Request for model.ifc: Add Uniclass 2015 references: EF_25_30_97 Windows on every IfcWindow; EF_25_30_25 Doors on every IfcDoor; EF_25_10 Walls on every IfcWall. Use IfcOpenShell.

First a look at what the model holds.

```python
import ifcopenshell

model = ifcopenshell.open("model.ifc")
print(model.schema)
print("classifications:", [c.Name for c in model.by_type("IfcClassification")])
for ifc_class in ("IfcDoor", "IfcRoof", "IfcStair", "IfcWall", "IfcWindow"):
    print(ifc_class, len(model.by_type(ifc_class)))
```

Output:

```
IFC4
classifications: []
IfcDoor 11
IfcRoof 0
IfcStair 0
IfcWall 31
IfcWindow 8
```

```python
import ifcopenshell
import ifcopenshell.api.classification

model = ifcopenshell.open("model.ifc")

system = ifcopenshell.api.classification.add_classification(model, classification="Uniclass 2015")

codes = {
    "IfcWindow": ("EF_25_30_97", "Windows"),
    "IfcDoor": ("EF_25_30_25", "Doors"),
    "IfcWall": ("EF_25_10", "Walls"),
}
for ifc_class, (code, name) in codes.items():
    products = model.by_type(ifc_class)
    ifcopenshell.api.classification.add_reference(
        model, products=products, classification=system, identification=code, name=name
    )
    print(code, len(products))

model.write("model_updated.ifc")
```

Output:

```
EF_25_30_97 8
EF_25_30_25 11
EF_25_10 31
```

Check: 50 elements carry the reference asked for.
